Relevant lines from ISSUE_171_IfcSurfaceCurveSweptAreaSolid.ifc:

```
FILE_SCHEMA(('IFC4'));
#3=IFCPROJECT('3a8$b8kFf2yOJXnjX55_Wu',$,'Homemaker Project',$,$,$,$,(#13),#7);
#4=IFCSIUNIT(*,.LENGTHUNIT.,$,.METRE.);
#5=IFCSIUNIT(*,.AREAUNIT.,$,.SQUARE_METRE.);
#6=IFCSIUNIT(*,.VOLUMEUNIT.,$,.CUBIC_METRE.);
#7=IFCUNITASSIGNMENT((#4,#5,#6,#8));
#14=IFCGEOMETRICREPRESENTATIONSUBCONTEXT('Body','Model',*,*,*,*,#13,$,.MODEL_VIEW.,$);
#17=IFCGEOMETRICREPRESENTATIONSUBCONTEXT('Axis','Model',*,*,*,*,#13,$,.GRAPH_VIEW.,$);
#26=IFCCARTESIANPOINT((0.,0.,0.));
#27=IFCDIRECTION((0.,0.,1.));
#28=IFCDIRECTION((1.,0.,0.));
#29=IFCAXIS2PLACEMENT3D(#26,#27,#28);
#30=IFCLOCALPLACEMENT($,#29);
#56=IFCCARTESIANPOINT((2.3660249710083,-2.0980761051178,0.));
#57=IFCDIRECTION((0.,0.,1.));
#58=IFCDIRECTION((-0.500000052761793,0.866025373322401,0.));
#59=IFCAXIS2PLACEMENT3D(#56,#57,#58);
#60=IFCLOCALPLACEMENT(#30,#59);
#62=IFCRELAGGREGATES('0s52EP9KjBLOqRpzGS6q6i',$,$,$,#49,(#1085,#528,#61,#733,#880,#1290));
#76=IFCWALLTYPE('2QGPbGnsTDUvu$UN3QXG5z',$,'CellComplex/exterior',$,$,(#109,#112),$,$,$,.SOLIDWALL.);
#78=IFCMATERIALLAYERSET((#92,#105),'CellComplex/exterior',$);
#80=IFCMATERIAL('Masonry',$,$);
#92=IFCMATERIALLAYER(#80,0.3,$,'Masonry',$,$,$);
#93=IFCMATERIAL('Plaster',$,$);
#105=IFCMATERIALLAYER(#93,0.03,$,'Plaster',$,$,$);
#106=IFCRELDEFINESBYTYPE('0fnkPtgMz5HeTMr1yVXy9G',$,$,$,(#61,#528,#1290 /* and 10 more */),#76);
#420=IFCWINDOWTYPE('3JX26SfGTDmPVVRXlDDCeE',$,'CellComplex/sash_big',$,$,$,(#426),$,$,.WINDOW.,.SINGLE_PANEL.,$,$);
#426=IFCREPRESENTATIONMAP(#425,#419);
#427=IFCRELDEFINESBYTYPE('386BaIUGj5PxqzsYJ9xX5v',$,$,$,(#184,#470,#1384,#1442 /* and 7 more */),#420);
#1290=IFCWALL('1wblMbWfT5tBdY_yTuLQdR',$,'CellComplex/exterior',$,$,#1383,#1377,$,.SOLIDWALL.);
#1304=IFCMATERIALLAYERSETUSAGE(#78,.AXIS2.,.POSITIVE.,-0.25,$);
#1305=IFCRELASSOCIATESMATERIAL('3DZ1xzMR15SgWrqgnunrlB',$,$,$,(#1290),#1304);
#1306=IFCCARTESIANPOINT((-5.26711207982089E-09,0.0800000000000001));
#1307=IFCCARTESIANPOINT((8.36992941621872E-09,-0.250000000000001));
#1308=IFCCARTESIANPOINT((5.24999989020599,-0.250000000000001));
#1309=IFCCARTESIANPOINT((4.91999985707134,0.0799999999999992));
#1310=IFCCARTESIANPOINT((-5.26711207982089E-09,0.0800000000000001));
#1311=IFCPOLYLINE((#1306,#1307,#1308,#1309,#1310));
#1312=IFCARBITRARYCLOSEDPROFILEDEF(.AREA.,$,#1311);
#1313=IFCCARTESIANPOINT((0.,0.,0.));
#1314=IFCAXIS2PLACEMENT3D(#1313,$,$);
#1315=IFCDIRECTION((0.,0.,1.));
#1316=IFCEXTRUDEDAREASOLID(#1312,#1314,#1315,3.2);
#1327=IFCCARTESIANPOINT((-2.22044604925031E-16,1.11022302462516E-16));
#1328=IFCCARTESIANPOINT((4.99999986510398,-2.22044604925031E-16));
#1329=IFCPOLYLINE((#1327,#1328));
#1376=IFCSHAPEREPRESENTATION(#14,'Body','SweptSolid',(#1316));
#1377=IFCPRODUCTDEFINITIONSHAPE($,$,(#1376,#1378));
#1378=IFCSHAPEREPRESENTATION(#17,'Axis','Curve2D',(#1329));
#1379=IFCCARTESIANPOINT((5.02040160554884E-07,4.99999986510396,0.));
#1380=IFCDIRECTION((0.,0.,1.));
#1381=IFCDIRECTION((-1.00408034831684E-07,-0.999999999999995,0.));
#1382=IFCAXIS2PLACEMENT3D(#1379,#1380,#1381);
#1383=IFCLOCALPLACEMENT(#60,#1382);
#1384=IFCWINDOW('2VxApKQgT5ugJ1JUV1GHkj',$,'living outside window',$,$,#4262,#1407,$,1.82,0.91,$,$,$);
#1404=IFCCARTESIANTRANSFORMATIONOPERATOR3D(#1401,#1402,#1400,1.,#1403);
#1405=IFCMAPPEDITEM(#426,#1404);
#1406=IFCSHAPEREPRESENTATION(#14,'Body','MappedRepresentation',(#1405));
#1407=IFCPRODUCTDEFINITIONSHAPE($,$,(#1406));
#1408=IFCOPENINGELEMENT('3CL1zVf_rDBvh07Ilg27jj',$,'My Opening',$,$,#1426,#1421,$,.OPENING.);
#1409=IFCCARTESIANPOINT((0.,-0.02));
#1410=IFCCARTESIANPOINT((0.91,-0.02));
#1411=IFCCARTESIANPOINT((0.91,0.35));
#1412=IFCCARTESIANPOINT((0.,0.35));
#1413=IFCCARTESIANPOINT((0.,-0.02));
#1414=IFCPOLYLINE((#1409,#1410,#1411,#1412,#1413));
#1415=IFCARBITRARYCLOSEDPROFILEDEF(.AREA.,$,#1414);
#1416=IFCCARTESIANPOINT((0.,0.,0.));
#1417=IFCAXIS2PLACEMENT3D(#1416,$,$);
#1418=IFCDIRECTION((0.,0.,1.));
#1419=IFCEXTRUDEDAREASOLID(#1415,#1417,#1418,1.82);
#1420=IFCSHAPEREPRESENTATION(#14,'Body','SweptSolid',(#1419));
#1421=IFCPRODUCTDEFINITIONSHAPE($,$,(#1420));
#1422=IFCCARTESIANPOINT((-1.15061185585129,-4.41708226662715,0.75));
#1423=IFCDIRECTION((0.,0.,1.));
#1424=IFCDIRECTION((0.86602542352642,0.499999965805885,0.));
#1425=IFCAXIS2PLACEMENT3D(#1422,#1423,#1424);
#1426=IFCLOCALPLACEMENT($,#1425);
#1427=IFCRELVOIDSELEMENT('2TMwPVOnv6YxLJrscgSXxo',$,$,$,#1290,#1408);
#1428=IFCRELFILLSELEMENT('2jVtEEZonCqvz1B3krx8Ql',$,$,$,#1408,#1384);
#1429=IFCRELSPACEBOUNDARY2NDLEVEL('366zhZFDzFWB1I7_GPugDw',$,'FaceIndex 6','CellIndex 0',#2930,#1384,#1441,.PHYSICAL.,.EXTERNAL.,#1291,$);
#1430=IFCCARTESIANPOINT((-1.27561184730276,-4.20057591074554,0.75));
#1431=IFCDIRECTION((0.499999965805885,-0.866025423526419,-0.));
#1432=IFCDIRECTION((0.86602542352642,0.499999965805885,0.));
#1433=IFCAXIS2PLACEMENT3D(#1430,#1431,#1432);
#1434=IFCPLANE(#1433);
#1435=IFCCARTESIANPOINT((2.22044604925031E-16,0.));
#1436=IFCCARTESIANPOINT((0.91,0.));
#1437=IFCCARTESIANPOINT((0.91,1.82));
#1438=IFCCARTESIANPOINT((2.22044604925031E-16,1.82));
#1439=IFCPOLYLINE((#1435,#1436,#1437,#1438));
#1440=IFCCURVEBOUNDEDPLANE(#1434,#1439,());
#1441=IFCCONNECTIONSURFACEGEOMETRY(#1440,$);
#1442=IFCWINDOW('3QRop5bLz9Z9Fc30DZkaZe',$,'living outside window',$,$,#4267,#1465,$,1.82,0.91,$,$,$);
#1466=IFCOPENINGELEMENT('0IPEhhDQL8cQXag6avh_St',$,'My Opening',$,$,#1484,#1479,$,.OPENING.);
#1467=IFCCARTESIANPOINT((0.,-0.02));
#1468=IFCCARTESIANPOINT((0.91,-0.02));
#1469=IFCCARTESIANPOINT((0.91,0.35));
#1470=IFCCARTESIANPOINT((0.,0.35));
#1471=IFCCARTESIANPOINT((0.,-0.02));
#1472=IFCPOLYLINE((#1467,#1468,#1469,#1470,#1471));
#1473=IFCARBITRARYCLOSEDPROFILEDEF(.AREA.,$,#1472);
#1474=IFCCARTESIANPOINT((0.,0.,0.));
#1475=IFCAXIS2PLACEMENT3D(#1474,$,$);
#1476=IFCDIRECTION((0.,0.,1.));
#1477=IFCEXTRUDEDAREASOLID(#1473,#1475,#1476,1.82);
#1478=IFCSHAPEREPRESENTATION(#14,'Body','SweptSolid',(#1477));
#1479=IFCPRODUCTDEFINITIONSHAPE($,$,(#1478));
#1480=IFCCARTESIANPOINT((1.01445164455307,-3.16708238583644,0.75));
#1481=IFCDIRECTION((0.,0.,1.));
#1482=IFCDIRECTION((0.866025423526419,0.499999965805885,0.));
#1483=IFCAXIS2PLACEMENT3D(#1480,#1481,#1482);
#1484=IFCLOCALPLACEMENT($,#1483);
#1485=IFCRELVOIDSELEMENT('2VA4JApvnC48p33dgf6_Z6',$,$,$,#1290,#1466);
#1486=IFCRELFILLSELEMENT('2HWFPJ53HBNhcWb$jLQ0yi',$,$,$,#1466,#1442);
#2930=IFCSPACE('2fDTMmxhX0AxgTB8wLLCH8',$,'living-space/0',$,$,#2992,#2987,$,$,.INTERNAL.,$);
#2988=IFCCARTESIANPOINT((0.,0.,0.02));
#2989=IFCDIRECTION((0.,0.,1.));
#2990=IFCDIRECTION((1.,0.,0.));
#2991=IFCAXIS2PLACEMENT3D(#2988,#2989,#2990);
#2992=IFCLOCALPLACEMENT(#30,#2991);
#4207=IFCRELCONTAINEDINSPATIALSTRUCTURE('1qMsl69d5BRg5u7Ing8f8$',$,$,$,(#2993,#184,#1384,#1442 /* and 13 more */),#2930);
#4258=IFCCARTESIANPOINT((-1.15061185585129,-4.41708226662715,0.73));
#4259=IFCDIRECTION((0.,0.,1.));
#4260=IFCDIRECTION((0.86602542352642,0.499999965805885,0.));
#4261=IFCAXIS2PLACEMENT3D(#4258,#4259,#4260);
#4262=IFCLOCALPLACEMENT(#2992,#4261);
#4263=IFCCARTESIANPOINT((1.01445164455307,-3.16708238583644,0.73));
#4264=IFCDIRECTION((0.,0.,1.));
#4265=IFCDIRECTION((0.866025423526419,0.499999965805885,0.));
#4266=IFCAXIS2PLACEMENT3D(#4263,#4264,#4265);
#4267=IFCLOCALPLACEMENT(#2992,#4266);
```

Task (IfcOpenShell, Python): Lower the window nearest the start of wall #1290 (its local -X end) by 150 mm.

```python
import numpy as np
import ifcopenshell
import ifcopenshell.api.geometry
import ifcopenshell.util.placement
import ifcopenshell.util.unit

model = ifcopenshell.open("ISSUE_171_IfcSurfaceCurveSweptAreaSolid.ifc")
unit_scale = ifcopenshell.util.unit.calculate_unit_scale(model)

window = model.by_guid("2VxApKQgT5ugJ1JUV1GHkj")
opening = window.FillsVoids[0].RelatingOpeningElement
dz = -0.15

shift = np.array([0.0, 0.0, dz])
# The window is not placed relative to its opening, so move both.
for product in (opening, window):
    matrix = ifcopenshell.util.placement.get_local_placement(product.ObjectPlacement)
    matrix[:3, 3] += shift
    ifcopenshell.api.geometry.edit_object_placement(model, product=product, matrix=matrix, is_si=False)

# Space boundary surfaces are stored in each space's coordinates; move them too.
for rel in window.ProvidesBoundaries:
    if not rel.ConnectionGeometry:
        continue
    surface = rel.ConnectionGeometry.SurfaceOnRelatingElement.BasisSurface
    space_matrix = ifcopenshell.util.placement.get_local_placement(rel.RelatingSpace.ObjectPlacement)
    point = np.array(surface.Position.Location.Coordinates) + space_matrix[:3, :3].T @ shift
    surface.Position = model.createIfcAxis2Placement3D(
        model.createIfcCartesianPoint(point.tolist()), surface.Position.Axis, surface.Position.RefDirection
    )

print(f"moved by {dz * unit_scale:+.3f} m")

model.write("ISSUE_171_IfcSurfaceCurveSweptAreaSolid-out.ifc")
```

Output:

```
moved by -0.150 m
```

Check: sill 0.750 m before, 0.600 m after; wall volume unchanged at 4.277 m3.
